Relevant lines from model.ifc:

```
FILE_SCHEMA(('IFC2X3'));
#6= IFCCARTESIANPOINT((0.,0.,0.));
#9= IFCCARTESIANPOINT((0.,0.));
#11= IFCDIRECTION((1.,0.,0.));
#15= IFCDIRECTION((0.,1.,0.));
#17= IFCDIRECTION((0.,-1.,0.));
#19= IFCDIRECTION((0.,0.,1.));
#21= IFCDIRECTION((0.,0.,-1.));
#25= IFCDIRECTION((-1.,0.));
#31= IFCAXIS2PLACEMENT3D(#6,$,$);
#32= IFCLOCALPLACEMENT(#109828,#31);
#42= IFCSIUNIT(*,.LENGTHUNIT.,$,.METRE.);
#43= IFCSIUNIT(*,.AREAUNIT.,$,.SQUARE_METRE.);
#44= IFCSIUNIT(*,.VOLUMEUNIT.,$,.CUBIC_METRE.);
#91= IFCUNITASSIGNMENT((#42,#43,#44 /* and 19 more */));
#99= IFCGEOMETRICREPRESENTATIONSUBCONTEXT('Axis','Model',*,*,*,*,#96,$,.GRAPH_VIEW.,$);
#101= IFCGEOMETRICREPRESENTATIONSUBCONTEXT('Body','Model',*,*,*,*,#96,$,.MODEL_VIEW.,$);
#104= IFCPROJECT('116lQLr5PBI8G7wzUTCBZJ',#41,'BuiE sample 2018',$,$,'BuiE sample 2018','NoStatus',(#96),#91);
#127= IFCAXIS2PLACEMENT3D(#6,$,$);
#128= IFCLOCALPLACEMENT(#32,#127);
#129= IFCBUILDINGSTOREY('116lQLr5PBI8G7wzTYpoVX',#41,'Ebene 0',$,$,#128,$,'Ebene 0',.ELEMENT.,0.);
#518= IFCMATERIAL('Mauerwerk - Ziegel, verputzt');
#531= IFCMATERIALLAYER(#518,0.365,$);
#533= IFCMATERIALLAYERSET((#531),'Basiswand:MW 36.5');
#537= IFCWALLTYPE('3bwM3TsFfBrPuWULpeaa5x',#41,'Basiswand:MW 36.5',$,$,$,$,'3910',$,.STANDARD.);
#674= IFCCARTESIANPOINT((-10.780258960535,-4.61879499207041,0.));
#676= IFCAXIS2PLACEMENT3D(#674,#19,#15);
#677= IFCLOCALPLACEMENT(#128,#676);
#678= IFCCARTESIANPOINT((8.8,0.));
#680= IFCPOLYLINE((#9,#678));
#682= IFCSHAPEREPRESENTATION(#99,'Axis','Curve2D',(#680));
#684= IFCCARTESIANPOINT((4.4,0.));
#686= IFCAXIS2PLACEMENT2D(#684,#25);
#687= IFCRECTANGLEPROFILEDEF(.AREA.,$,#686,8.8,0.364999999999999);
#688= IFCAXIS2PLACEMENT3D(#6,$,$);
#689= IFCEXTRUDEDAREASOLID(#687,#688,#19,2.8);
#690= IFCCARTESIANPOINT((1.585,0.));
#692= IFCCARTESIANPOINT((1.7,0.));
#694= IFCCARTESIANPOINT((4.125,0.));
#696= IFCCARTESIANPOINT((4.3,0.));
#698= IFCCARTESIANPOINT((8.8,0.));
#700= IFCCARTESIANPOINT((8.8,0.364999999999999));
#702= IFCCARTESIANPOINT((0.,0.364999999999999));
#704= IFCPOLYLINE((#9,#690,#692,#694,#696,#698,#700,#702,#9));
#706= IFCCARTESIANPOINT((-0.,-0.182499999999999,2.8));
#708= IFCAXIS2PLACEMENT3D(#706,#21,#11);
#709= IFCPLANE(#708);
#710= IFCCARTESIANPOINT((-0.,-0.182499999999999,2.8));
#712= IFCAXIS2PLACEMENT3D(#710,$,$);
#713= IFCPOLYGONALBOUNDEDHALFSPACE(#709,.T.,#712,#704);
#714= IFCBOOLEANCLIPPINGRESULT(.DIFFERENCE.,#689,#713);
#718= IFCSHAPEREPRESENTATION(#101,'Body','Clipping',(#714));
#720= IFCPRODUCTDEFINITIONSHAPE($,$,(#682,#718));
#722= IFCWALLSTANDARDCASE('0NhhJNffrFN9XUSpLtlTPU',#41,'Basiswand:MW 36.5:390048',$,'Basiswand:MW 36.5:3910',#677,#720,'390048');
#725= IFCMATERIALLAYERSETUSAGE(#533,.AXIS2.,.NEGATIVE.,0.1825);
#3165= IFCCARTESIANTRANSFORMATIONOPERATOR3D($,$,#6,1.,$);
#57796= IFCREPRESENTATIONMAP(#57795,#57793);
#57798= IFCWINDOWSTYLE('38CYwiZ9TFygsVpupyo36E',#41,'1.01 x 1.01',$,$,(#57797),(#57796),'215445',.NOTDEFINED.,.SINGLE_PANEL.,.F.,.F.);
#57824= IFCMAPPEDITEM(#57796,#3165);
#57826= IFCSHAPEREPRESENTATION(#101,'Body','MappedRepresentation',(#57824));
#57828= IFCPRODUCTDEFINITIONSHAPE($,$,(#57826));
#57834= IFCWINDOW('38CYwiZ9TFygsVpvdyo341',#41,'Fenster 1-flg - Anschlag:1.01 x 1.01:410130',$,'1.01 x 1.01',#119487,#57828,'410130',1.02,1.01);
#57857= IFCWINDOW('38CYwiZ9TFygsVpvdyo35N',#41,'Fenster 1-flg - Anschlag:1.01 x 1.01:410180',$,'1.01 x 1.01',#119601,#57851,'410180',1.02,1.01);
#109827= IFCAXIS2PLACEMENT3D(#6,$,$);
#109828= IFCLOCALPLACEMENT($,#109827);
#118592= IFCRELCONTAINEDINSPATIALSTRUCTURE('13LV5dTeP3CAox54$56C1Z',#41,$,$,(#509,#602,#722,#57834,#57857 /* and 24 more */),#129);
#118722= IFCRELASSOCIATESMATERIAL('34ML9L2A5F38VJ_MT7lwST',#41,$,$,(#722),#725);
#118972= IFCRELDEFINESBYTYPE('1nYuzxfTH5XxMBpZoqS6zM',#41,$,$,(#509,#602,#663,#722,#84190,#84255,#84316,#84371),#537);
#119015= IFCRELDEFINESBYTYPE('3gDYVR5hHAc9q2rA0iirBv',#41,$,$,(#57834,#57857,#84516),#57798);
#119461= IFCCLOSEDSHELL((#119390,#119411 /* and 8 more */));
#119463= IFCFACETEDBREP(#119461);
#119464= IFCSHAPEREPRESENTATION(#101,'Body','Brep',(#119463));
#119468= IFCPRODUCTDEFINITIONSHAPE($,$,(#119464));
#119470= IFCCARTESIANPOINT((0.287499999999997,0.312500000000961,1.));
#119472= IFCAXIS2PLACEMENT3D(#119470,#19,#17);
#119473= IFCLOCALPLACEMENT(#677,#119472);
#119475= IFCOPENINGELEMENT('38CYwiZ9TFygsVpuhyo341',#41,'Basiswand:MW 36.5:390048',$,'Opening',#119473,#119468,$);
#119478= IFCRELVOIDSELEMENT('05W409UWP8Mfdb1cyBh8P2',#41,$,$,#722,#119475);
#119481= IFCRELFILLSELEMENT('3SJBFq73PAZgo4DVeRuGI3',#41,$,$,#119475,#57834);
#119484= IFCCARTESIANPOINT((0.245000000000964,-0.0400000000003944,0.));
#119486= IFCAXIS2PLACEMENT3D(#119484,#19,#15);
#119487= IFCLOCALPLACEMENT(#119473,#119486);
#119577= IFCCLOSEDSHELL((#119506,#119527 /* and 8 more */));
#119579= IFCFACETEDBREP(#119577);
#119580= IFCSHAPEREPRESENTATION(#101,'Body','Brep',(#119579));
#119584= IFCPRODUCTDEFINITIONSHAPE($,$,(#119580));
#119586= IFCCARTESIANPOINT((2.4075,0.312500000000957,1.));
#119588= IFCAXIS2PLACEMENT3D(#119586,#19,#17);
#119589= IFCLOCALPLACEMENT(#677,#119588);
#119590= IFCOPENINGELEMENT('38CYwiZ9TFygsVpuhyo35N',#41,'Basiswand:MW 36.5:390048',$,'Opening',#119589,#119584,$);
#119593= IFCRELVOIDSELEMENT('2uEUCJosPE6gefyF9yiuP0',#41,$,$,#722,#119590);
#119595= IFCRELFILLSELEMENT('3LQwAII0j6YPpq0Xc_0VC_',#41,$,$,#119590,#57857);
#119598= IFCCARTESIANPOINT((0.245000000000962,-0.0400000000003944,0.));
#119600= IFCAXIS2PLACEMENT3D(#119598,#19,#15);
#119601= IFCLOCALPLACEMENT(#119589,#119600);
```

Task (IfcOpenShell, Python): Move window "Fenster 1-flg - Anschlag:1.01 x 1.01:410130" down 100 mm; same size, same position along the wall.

```python
import numpy as np
import ifcopenshell
import ifcopenshell.api.geometry
import ifcopenshell.util.placement
import ifcopenshell.util.unit

model = ifcopenshell.open("model.ifc")
unit_scale = ifcopenshell.util.unit.calculate_unit_scale(model)

window = model.by_id(57834)
opening = window.FillsVoids[0].RelatingOpeningElement
dz = -0.1 / unit_scale

shift = np.array([0.0, 0.0, dz])
# The window is placed relative to its opening, so it follows when the opening moves.
matrix = ifcopenshell.util.placement.get_local_placement(opening.ObjectPlacement)
matrix[:3, 3] += shift
ifcopenshell.api.geometry.edit_object_placement(
    model, product=opening, matrix=matrix, is_si=False, should_transform_children=True
)

print(f"moved by {dz * unit_scale:+.3f} m")

model.write("model_updated.ifc")
```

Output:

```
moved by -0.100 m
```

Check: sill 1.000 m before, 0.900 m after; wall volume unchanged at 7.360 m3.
